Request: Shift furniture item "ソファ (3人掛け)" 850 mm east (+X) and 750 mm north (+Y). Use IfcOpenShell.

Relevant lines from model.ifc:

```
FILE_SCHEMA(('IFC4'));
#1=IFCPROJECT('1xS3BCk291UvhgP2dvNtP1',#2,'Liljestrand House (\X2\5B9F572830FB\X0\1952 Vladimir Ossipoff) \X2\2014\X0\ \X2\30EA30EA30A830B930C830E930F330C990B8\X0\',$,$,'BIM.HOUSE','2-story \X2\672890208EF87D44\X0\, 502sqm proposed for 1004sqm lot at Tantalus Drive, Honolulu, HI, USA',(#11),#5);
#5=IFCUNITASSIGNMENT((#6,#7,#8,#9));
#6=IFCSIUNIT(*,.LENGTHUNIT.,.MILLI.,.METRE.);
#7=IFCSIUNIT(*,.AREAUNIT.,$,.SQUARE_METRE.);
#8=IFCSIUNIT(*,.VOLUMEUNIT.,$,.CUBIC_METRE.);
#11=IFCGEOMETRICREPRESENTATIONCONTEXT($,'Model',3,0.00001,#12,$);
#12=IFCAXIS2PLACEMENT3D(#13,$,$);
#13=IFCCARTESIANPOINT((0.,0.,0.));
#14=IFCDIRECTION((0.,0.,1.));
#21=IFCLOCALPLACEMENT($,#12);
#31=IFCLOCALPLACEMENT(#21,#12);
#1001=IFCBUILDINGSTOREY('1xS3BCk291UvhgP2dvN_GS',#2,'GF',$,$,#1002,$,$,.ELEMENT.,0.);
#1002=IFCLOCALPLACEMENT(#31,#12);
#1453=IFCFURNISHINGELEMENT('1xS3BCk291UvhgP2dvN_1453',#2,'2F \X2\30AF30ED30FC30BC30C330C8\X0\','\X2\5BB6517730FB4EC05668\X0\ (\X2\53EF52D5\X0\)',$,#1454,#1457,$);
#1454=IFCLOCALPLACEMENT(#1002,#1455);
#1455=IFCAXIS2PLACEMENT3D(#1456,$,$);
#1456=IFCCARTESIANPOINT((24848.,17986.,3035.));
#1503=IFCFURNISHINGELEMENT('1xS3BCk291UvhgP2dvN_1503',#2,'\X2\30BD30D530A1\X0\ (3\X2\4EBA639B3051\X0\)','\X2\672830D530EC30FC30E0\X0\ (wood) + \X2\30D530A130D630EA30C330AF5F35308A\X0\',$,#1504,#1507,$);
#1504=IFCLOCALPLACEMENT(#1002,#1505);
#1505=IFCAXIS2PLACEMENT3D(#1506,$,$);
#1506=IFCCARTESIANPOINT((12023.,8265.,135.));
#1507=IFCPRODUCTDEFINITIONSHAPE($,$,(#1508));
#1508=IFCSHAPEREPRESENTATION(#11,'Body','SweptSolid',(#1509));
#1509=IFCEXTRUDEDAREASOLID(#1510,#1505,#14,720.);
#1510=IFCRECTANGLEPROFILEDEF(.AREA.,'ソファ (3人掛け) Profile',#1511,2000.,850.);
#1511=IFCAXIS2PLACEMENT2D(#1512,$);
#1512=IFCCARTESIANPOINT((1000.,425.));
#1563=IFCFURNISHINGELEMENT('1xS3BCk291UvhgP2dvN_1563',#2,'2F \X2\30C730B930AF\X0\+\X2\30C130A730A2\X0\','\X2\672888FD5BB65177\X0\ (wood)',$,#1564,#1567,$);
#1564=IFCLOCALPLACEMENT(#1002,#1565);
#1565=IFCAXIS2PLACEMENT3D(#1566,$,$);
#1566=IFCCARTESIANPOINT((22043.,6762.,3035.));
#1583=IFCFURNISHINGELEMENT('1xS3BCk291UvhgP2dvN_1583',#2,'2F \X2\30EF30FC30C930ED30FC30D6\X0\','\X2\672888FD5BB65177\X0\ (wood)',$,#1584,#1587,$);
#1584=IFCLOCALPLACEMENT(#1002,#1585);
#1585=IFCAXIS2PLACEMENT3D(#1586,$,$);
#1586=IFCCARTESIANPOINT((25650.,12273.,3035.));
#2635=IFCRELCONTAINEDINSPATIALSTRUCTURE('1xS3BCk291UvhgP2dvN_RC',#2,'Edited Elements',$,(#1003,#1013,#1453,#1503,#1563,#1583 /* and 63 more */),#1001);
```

```python
import ifcopenshell
import ifcopenshell.api.geometry
import ifcopenshell.util.placement

model = ifcopenshell.open("model.ifc")

item = model.by_guid("1xS3BCk291UvhgP2dvN_1503")
matrix = ifcopenshell.util.placement.get_local_placement(item.ObjectPlacement)
matrix[0, 3] += 850.0
matrix[1, 3] += 750.0
ifcopenshell.api.geometry.edit_object_placement(model, product=item, matrix=matrix, is_si=False)

print(ifcopenshell.util.placement.get_local_placement(item.ObjectPlacement).round(3) + 0.0)

model.write("model_rev.ifc")
```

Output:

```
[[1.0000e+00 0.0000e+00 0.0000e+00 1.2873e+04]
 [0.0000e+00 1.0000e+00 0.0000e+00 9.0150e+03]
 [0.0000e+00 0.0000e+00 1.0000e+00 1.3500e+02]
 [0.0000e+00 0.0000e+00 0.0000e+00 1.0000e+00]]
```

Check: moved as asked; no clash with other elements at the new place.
